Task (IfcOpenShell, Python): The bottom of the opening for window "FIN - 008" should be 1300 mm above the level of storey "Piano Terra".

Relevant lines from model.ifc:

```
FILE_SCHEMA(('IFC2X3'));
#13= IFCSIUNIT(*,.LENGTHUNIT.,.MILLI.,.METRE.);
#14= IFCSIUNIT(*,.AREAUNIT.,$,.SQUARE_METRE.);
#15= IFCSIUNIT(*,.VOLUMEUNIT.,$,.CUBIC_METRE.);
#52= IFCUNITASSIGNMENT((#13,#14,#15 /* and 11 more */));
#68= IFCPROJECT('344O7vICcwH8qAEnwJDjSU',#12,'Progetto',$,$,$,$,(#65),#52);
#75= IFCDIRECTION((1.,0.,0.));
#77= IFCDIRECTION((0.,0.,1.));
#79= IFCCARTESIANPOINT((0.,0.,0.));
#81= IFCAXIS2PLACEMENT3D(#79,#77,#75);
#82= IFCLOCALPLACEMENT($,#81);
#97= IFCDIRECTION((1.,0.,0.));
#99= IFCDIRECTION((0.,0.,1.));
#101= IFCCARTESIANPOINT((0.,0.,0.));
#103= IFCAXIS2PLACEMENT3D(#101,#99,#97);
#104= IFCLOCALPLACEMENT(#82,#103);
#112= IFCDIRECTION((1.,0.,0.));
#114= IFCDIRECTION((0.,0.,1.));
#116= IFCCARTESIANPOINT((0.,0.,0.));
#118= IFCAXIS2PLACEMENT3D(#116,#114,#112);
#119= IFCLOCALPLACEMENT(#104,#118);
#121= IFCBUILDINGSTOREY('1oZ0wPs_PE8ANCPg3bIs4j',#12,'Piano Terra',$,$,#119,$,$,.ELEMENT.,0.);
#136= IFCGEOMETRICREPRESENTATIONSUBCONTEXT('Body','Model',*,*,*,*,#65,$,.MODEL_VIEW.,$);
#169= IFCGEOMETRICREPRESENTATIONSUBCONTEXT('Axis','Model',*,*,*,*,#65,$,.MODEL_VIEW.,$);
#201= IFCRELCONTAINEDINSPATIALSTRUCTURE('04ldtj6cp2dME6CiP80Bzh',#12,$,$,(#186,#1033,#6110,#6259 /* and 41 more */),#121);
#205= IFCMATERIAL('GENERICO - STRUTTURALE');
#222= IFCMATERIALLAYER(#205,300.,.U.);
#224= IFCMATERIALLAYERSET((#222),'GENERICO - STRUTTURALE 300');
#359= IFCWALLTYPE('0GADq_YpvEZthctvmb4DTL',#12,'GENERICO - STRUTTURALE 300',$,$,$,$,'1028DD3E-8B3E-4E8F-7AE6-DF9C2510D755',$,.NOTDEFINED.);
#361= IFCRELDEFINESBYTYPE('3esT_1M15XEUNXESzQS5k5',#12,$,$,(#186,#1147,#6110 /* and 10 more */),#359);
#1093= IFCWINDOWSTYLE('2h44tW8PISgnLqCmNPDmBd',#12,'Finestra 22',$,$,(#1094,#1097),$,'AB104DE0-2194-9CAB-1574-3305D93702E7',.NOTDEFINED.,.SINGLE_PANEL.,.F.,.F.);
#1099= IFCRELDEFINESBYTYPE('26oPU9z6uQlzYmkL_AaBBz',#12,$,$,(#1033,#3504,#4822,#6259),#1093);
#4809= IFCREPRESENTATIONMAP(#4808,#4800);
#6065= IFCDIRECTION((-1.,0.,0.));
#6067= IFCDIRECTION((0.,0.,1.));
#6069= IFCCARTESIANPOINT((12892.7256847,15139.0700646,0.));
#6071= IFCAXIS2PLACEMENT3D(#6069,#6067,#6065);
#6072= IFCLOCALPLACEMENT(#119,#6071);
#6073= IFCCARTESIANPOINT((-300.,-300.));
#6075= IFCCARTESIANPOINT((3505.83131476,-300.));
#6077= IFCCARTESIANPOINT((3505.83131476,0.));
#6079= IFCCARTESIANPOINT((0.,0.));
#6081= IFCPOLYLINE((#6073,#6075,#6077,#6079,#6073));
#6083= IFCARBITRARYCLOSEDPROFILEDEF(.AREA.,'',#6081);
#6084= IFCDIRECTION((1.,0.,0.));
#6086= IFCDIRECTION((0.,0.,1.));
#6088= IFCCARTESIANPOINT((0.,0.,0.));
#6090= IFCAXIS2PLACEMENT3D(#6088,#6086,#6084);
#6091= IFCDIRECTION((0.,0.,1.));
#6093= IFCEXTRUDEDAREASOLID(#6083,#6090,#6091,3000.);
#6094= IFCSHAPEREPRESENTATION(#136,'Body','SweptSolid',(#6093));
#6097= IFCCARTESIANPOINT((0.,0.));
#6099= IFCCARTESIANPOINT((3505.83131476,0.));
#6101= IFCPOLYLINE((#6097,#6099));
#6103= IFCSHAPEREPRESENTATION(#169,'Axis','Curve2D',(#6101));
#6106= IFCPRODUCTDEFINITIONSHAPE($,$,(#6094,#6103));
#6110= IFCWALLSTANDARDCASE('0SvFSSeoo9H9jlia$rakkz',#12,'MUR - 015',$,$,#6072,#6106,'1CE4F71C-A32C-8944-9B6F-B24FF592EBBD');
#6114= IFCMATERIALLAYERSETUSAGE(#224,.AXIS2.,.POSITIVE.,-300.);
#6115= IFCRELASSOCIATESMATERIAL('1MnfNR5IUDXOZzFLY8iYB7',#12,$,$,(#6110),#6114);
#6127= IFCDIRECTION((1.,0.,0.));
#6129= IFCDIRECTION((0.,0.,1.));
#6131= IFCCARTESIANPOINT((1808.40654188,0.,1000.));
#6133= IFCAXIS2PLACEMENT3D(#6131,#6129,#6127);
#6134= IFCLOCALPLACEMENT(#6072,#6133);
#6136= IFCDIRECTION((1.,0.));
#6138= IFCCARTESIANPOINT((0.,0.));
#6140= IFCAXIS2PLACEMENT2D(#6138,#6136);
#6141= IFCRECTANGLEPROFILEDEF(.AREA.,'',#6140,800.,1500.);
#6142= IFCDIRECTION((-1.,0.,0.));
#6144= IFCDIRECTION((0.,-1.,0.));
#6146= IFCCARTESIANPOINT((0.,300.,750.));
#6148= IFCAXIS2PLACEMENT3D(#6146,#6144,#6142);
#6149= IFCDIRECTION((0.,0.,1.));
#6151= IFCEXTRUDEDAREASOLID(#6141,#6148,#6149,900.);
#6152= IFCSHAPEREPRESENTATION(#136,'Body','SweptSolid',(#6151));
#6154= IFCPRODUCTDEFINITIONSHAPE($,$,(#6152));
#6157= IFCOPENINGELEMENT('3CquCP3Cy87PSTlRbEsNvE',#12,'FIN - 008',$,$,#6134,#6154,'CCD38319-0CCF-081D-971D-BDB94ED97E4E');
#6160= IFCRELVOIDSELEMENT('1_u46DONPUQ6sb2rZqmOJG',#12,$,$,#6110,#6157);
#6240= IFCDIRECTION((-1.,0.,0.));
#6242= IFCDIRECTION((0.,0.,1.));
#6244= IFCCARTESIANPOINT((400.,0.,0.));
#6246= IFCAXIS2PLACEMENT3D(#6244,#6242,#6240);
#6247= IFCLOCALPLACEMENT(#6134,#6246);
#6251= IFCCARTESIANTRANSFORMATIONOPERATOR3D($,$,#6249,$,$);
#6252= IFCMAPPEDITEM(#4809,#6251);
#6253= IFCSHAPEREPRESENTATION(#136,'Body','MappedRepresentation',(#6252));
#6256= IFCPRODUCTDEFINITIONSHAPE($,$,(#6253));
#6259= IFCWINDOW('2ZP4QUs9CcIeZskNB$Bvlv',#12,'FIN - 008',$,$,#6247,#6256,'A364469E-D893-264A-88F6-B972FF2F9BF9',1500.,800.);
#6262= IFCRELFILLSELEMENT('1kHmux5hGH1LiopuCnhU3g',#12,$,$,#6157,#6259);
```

```python
import numpy as np
import ifcopenshell
import ifcopenshell.api.geometry
import ifcopenshell.geom
import ifcopenshell.util.element
import ifcopenshell.util.placement
import ifcopenshell.util.shape
import ifcopenshell.util.unit

model = ifcopenshell.open("model.ifc")
unit_scale = ifcopenshell.util.unit.calculate_unit_scale(model)

window = model.by_id(6259)
opening = window.FillsVoids[0].RelatingOpeningElement
storey = ifcopenshell.util.element.get_container(window, ifc_class="IfcBuildingStorey")
level = ifcopenshell.util.placement.get_local_placement(storey.ObjectPlacement)[2, 3]

# The opening's origin need not be at the sill, so measure its lowest point.
shape = ifcopenshell.geom.create_shape(ifcopenshell.geom.settings(), opening)
bottom = ifcopenshell.util.shape.get_shape_bottom_elevation(shape, shape.geometry) / unit_scale
dz = level + 1.3 / unit_scale - bottom

shift = np.array([0.0, 0.0, dz])
# The window is placed relative to its opening, so it follows when the opening moves.
matrix = ifcopenshell.util.placement.get_local_placement(opening.ObjectPlacement)
matrix[:3, 3] += shift
ifcopenshell.api.geometry.edit_object_placement(
    model, product=opening, matrix=matrix, is_si=False, should_transform_children=True
)

print(f"moved by {dz * unit_scale:+.3f} m")

model.write("model_v2.ifc")
```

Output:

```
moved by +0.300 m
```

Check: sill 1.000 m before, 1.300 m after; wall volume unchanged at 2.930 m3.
